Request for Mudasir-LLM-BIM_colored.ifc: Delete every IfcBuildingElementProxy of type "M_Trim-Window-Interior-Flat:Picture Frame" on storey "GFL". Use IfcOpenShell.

First a look at what the model holds.

```python
import ifcopenshell
import ifcopenshell.util.element

model = ifcopenshell.open("Mudasir-LLM-BIM_colored.ifc")
print(model.schema)
storey = next(s for s in model.by_type("IfcBuildingStorey") if s.Name == "GFL")
proxies = [e for e in ifcopenshell.util.element.get_decomposition(storey) if e.is_a("IfcBuildingElementProxy")]
seen = {}
for e in proxies:
    element_type = ifcopenshell.util.element.get_type(e)
    name = element_type.Name if element_type not in (None, e) else None
    seen[name] = seen.get(name, 0) + 1
for name, count in sorted(seen.items(), key=str):
    print(count, "x", name)
```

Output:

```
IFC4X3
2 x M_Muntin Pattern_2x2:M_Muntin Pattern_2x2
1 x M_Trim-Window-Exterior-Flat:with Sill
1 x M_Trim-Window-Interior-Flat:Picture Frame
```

```python
import ifcopenshell
import ifcopenshell.api.root
import ifcopenshell.util.element

model = ifcopenshell.open("Mudasir-LLM-BIM_colored.ifc")

storey = next(s for s in model.by_type("IfcBuildingStorey") if s.Name == "GFL")
proxies = [e for e in ifcopenshell.util.element.get_decomposition(storey) if e.is_a("IfcBuildingElementProxy")]
targets = [e for e in proxies if (t := ifcopenshell.util.element.get_type(e)) not in (None, e) and t.Name == "M_Trim-Window-Interior-Flat:Picture Frame"]

for e in targets:
    ifcopenshell.api.root.remove_product(model, product=e)
print(len(targets), "removed")

model.write("Mudasir-LLM-BIM_colored_rev.ifc")
```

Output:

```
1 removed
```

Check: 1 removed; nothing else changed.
